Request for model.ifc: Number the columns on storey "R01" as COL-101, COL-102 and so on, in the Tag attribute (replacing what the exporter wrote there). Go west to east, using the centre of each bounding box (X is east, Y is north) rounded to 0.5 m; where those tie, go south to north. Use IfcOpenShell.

First a look at what the model holds.

```python
import ifcopenshell
import ifcopenshell.util.element
import ifcopenshell.util.placement

model = ifcopenshell.open("model.ifc")
print(model.schema)
storey = next(s for s in model.by_type("IfcBuildingStorey") if s.Name == "R01")
columns = [e for e in ifcopenshell.util.element.get_decomposition(storey) if e.is_a("IfcColumn")]
for e in sorted(columns, key=lambda e: e.id()):
    origin = ifcopenshell.util.placement.get_local_placement(e.ObjectPlacement)[:3, 3]
    print(e.id(), e.Tag, e.Name, origin.round(2) + 0.0, sep=" | ")
```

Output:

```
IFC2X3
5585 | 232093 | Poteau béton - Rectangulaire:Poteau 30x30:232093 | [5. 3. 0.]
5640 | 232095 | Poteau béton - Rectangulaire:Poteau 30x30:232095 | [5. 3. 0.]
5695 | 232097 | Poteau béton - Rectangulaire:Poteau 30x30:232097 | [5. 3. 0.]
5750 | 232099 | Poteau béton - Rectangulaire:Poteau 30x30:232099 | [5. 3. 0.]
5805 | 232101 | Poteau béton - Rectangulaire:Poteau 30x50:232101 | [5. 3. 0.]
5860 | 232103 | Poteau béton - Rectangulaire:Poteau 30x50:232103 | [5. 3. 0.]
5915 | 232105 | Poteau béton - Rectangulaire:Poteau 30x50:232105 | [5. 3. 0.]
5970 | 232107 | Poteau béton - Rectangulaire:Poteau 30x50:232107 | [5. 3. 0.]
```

```python
import ifcopenshell
import ifcopenshell.geom
import ifcopenshell.util.element
import ifcopenshell.util.shape

model = ifcopenshell.open("model.ifc")
settings = ifcopenshell.geom.settings()
settings.set("use-world-coords", True)


def centre(element):
    shape = ifcopenshell.geom.create_shape(settings, element)
    return ifcopenshell.util.shape.get_bbox_centroid(shape.geometry)


storey = next(s for s in model.by_type("IfcBuildingStorey") if s.Name == "R01")
columns = [e for e in ifcopenshell.util.element.get_decomposition(storey) if e.is_a("IfcColumn")]

# Insertion points can sit at a corner or the storey origin, so sort by the geometry (in metres).
centres = {e: centre(e) for e in columns}
columns.sort(key=lambda e: (round(centres[e][0] / 0.5), centres[e][1]))

for i, e in enumerate(columns, start=1):
    number = f"COL-1{i:02d}"
    e.Tag = number
    print(e.id(), number)

model.write("model_edited.ifc")
```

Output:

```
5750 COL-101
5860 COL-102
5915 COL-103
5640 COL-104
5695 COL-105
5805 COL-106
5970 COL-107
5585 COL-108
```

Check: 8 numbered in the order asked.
